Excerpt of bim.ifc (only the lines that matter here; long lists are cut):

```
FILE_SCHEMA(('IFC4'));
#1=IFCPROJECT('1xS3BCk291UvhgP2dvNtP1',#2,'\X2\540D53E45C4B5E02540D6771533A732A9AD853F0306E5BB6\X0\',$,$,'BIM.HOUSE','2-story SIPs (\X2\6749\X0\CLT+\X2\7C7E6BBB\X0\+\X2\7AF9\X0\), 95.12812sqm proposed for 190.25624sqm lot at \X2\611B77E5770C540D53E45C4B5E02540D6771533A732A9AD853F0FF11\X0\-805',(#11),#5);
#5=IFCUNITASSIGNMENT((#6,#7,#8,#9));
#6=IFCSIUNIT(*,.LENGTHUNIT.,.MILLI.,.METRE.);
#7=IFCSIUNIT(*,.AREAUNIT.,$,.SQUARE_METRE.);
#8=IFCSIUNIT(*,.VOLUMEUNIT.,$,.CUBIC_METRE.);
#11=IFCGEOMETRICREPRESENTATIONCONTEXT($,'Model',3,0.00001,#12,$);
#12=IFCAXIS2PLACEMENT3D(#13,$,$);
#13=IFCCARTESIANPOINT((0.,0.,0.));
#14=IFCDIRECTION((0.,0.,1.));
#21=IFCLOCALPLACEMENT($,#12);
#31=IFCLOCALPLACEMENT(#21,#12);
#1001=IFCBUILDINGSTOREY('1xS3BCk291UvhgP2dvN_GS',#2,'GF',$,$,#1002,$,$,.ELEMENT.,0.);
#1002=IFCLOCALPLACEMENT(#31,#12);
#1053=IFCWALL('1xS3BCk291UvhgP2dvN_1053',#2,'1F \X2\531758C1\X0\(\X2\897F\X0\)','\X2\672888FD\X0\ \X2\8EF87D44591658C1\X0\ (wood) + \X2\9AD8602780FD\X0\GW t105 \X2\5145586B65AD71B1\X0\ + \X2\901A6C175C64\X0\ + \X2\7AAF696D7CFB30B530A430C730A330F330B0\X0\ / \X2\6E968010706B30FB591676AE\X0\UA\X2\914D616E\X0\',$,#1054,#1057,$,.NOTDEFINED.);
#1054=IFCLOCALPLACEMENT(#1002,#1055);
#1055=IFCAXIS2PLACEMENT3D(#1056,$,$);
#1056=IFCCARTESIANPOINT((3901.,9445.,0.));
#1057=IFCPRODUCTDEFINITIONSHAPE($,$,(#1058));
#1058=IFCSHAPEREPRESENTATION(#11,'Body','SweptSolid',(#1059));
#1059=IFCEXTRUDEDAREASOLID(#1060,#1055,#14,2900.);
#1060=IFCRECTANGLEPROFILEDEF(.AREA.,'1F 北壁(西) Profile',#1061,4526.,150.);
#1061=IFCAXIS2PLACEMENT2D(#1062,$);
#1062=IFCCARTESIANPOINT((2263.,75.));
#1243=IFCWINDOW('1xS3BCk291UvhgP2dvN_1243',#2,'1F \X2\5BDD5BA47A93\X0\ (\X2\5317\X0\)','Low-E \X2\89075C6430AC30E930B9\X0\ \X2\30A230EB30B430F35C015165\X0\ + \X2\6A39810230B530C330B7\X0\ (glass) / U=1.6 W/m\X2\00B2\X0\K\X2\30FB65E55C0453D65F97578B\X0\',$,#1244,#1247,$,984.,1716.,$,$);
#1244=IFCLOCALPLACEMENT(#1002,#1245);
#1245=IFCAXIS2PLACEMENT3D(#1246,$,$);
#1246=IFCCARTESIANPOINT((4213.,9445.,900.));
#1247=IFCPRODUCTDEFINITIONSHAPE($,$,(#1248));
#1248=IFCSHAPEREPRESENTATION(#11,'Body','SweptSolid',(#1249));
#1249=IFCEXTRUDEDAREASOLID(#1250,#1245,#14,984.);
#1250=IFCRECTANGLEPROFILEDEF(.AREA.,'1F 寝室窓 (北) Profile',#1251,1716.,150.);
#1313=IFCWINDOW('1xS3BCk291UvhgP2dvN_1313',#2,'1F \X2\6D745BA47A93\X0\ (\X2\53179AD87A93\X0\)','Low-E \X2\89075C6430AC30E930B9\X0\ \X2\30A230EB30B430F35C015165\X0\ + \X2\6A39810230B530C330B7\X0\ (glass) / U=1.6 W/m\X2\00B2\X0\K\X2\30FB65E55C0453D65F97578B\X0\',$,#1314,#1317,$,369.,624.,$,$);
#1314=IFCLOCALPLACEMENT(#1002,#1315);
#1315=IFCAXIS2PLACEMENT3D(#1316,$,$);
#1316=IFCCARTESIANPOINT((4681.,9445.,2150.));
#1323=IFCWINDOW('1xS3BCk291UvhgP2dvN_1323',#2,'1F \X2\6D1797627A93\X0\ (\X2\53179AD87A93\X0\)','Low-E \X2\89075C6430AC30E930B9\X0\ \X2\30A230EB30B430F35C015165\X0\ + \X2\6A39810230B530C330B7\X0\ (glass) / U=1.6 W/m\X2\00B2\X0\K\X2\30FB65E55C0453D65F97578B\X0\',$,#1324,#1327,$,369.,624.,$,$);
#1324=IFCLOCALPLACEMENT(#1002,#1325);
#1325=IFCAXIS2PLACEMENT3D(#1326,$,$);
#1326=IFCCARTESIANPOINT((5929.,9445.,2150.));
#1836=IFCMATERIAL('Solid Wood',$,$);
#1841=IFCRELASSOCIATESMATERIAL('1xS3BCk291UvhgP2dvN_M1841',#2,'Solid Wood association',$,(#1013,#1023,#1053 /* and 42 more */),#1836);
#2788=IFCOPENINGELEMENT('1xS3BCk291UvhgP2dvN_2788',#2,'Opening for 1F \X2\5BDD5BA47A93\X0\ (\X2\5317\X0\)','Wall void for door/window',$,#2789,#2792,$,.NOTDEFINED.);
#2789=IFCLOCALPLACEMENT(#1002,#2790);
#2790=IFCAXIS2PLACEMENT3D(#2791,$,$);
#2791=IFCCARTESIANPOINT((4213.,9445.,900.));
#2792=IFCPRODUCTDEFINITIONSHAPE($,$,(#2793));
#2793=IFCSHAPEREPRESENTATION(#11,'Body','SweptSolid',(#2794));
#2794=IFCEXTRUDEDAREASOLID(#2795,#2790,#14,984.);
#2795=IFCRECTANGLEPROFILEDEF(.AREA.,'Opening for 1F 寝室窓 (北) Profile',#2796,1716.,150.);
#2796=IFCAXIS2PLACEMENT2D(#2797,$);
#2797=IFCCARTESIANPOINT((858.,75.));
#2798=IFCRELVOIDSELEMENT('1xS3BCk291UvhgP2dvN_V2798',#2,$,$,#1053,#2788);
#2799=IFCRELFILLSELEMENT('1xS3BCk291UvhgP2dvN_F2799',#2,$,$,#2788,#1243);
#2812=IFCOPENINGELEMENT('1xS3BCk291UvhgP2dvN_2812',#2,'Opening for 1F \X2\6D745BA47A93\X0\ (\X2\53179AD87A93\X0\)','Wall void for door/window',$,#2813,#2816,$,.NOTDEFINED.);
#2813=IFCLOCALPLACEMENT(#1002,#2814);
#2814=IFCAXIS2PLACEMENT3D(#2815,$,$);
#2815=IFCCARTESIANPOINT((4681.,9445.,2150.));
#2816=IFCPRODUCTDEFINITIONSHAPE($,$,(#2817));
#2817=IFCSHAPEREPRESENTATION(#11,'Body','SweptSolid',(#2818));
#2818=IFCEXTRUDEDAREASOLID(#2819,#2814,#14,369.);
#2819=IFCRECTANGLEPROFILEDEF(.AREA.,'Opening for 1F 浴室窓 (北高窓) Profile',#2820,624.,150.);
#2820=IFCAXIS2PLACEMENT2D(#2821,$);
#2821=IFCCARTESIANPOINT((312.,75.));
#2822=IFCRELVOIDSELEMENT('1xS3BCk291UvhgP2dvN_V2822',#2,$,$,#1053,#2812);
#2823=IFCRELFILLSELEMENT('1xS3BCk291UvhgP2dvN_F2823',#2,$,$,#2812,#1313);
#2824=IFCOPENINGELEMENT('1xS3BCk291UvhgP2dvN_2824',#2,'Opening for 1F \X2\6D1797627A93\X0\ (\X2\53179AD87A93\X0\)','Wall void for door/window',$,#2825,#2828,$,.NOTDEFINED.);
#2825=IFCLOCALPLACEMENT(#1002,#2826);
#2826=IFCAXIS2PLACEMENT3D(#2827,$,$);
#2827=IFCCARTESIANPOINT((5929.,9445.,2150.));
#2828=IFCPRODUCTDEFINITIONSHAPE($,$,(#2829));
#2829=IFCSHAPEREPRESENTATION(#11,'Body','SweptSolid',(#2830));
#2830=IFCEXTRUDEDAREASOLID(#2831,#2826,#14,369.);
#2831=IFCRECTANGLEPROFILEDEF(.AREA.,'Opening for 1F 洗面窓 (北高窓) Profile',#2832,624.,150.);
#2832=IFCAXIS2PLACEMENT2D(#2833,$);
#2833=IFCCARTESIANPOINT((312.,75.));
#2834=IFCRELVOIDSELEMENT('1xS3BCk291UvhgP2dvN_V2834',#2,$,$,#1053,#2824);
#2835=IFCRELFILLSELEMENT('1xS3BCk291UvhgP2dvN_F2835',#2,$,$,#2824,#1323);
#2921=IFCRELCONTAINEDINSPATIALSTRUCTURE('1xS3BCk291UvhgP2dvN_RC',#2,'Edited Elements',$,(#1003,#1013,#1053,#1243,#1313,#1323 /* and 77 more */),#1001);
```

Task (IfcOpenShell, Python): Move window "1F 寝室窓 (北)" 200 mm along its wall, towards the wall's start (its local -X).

```python
import ifcopenshell
import ifcopenshell.api.geometry
import ifcopenshell.util.placement

model = ifcopenshell.open("bim.ifc")

window = model.by_guid("1xS3BCk291UvhgP2dvN_1243")
opening = window.FillsVoids[0].RelatingOpeningElement
wall = opening.VoidsElements[0].RelatingBuildingElement

wall_matrix = ifcopenshell.util.placement.get_local_placement(wall.ObjectPlacement)
shift = wall_matrix[:3, 0] * -200.0
before = ifcopenshell.util.placement.get_local_placement(window.ObjectPlacement)[:3, 3].copy()

# The window is not placed relative to its opening, so move both.
for product in (opening, window):
    matrix = ifcopenshell.util.placement.get_local_placement(product.ObjectPlacement)
    matrix[:3, 3] += shift
    ifcopenshell.api.geometry.edit_object_placement(model, product=product, matrix=matrix, is_si=False)

after = ifcopenshell.util.placement.get_local_placement(window.ObjectPlacement)[:3, 3]
print("window moved by", (after - before).round(3) + 0.0)

model.write("bim_edited.ifc")
```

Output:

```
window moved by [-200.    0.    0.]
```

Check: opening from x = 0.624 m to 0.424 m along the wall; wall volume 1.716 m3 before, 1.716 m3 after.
